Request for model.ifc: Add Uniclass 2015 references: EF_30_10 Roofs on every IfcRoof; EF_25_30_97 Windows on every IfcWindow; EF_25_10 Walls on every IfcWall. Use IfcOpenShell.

First a look at what the model holds.

```python
import ifcopenshell

model = ifcopenshell.open("model.ifc")
print(model.schema)
print("classifications:", [c.Name for c in model.by_type("IfcClassification")])
for ifc_class in ("IfcDoor", "IfcRoof", "IfcStair", "IfcWall", "IfcWindow"):
    print(ifc_class, len(model.by_type(ifc_class)))
```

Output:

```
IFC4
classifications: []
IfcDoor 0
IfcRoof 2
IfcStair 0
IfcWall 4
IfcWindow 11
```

```python
import ifcopenshell
import ifcopenshell.api.classification

model = ifcopenshell.open("model.ifc")

system = ifcopenshell.api.classification.add_classification(model, classification="Uniclass 2015")

codes = {
    "IfcRoof": ("EF_30_10", "Roofs"),
    "IfcWindow": ("EF_25_30_97", "Windows"),
    "IfcWall": ("EF_25_10", "Walls"),
}
for ifc_class, (code, name) in codes.items():
    products = model.by_type(ifc_class)
    ifcopenshell.api.classification.add_reference(
        model, products=products, classification=system, identification=code, name=name
    )
    print(code, len(products))

model.write("model_rev.ifc")
```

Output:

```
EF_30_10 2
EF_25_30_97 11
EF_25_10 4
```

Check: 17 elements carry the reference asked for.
